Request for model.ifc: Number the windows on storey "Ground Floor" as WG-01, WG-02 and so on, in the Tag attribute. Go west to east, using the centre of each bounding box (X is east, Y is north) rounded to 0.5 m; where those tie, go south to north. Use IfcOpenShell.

First a look at what the model holds.

```python
import ifcopenshell
import ifcopenshell.util.element
import ifcopenshell.util.placement

model = ifcopenshell.open("model.ifc")
print(model.schema)
storey = next(s for s in model.by_type("IfcBuildingStorey") if s.Name == "Ground Floor")
windows = [e for e in ifcopenshell.util.element.get_decomposition(storey) if e.is_a("IfcWindow")]
for e in sorted(windows, key=lambda e: e.id()):
    origin = ifcopenshell.util.placement.get_local_placement(e.ObjectPlacement)[:3, 3]
    print(e.id(), e.Tag, e.Name, origin.round(2) + 0.0, sep=" | ")
```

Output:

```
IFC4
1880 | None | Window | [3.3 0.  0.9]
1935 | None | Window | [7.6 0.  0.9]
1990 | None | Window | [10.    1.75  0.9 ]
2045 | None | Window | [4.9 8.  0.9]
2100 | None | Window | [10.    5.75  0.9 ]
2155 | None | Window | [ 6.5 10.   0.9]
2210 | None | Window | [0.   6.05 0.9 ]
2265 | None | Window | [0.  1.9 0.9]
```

```python
import ifcopenshell
import ifcopenshell.geom
import ifcopenshell.util.element
import ifcopenshell.util.shape

model = ifcopenshell.open("model.ifc")
settings = ifcopenshell.geom.settings()
settings.set("use-world-coords", True)


def centre(element):
    shape = ifcopenshell.geom.create_shape(settings, element)
    return ifcopenshell.util.shape.get_bbox_centroid(shape.geometry)


storey = next(s for s in model.by_type("IfcBuildingStorey") if s.Name == "Ground Floor")
windows = [e for e in ifcopenshell.util.element.get_decomposition(storey) if e.is_a("IfcWindow")]

# Insertion points can sit at a corner or the storey origin, so sort by the geometry (in metres).
centres = {e: centre(e) for e in windows}
windows.sort(key=lambda e: (round(centres[e][0] / 0.5), centres[e][1]))

for i, e in enumerate(windows, start=1):
    number = f"WG-{i:02d}"
    e.Tag = number
    print(e.id(), number)

model.write("model_v2.ifc")
```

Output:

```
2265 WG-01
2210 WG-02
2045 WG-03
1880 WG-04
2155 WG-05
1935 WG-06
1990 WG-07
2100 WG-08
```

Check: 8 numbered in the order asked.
